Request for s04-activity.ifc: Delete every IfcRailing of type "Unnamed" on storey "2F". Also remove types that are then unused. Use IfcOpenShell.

First a look at what the model holds.

```python
import ifcopenshell
import ifcopenshell.util.element

model = ifcopenshell.open("s04-activity.ifc")
print(model.schema)
storey = next(s for s in model.by_type("IfcBuildingStorey") if s.Name == "2F")
railings = [e for e in ifcopenshell.util.element.get_decomposition(storey) if e.is_a("IfcRailing")]
seen = {}
for e in railings:
    element_type = ifcopenshell.util.element.get_type(e)
    name = element_type.Name if element_type not in (None, e) else None
    seen[name] = seen.get(name, 0) + 1
for name, count in sorted(seen.items(), key=str):
    print(count, "x", name)
```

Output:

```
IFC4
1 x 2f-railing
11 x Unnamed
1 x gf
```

```python
import ifcopenshell
import ifcopenshell.api.root
import ifcopenshell.util.element

model = ifcopenshell.open("s04-activity.ifc")

storey = next(s for s in model.by_type("IfcBuildingStorey") if s.Name == "2F")
railings = [e for e in ifcopenshell.util.element.get_decomposition(storey) if e.is_a("IfcRailing")]
targets = [e for e in railings if (t := ifcopenshell.util.element.get_type(e)) not in (None, e) and t.Name == "Unnamed"]
types = {ifcopenshell.util.element.get_type(e) for e in targets} - {None, *targets}

for e in targets:
    ifcopenshell.api.root.remove_product(model, product=e)
print(len(targets), "removed")

unused = [t for t in types if not ifcopenshell.util.element.get_types(t)]
for t in unused:
    ifcopenshell.api.root.remove_product(model, product=t)
print(len(unused), "unused types removed")

model.write("s04-activity_edited.ifc")
```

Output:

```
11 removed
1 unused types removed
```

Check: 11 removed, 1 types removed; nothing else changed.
